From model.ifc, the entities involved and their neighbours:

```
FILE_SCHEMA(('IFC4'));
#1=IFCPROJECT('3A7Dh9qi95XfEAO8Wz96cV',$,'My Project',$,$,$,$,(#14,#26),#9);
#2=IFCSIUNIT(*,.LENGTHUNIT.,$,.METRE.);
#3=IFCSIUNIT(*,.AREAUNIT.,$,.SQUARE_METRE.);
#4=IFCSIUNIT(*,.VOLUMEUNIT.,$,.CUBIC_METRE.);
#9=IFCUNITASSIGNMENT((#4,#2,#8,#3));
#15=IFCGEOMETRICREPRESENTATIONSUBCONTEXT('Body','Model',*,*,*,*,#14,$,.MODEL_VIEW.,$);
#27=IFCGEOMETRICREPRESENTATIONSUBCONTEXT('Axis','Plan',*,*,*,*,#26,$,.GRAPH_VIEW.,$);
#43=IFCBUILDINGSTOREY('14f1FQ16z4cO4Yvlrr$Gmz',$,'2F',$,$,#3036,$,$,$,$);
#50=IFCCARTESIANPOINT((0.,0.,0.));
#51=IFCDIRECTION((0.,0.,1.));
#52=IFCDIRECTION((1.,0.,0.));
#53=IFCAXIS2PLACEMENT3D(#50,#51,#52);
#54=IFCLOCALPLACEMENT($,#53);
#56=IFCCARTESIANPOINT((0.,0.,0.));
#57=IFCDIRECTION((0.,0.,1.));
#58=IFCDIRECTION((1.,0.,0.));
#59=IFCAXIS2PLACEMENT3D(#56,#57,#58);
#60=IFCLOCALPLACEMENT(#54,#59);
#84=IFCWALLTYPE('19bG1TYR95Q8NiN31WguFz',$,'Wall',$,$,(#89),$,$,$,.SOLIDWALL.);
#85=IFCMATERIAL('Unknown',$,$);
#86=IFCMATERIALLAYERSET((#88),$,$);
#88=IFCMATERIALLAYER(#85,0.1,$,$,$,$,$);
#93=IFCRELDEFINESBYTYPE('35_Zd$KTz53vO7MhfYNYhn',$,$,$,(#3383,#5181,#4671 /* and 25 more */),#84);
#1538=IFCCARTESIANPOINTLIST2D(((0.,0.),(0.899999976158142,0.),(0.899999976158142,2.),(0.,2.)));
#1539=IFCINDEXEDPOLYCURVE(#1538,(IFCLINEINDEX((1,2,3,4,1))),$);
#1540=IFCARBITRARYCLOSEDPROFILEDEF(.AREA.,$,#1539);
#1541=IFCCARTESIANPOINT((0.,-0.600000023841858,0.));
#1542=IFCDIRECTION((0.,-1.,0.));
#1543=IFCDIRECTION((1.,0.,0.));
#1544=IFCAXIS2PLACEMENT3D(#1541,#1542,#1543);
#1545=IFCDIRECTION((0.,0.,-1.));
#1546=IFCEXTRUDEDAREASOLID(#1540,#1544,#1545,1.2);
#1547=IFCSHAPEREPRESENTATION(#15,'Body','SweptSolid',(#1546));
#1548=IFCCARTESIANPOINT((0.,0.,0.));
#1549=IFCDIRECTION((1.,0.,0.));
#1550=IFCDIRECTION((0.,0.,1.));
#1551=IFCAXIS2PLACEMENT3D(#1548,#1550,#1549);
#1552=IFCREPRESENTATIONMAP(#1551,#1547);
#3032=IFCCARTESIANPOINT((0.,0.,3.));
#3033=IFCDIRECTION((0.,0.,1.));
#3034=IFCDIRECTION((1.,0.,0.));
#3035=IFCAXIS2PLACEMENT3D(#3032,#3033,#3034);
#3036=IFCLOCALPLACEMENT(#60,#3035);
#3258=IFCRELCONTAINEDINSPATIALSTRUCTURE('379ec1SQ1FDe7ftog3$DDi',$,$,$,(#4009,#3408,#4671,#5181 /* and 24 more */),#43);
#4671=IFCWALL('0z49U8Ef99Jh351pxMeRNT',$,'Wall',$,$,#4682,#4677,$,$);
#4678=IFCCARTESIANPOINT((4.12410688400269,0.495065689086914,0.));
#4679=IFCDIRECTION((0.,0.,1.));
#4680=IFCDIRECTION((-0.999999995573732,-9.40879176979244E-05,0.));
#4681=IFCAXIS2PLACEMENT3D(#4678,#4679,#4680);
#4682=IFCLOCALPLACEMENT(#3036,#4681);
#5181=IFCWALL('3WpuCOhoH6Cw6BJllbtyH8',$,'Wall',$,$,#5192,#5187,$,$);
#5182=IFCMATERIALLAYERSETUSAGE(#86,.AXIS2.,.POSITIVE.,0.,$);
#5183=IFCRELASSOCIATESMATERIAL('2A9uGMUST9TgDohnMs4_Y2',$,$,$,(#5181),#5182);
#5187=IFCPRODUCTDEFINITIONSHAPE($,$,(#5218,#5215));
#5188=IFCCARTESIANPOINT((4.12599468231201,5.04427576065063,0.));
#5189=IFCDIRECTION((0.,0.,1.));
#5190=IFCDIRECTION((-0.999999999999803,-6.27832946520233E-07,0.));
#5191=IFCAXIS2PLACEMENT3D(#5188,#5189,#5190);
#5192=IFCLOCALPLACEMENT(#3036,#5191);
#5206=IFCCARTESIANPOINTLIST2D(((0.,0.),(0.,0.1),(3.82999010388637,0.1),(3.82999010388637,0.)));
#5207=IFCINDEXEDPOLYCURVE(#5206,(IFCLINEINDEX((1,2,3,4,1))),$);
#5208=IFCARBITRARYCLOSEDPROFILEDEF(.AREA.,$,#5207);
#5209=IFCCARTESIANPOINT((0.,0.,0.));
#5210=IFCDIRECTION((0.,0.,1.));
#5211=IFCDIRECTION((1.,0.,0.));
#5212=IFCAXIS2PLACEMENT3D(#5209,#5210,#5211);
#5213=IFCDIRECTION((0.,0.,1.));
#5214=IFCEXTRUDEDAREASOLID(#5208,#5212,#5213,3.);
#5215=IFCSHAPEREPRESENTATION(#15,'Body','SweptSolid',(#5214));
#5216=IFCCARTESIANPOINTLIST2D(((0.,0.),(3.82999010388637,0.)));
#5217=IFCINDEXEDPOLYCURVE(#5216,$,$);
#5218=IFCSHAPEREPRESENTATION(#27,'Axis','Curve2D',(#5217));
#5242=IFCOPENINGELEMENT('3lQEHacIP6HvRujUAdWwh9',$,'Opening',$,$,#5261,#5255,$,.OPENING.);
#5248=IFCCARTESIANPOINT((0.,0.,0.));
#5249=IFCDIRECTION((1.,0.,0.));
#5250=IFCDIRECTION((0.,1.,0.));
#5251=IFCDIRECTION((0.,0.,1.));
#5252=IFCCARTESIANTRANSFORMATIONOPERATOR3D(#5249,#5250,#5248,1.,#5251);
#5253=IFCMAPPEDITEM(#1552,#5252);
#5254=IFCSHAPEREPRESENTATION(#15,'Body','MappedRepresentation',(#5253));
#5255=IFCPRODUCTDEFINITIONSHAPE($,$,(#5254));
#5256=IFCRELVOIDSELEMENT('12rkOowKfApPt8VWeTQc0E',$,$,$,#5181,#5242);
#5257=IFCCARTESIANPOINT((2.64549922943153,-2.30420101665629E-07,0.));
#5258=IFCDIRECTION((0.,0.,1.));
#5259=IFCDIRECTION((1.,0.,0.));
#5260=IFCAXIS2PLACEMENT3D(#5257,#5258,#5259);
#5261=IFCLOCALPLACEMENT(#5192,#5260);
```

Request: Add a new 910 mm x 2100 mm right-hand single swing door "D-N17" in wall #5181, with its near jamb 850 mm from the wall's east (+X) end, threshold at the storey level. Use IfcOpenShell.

```python
import numpy as np
import ifcopenshell
import ifcopenshell.api.feature
import ifcopenshell.api.geometry
import ifcopenshell.api.root
import ifcopenshell.api.spatial
import ifcopenshell.geom
import ifcopenshell.util.element
import ifcopenshell.util.placement
import ifcopenshell.util.representation
import ifcopenshell.util.shape
import ifcopenshell.util.unit

model = ifcopenshell.open("model.ifc")
unit_scale = ifcopenshell.util.unit.calculate_unit_scale(model)
settings = ifcopenshell.geom.settings()


def volume(element):
    """Net volume in cubic metres, openings subtracted."""
    shape = ifcopenshell.geom.create_shape(settings, element)
    return ifcopenshell.util.shape.get_volume(shape.geometry)


wall = model.by_guid("3WpuCOhoH6Cw6BJllbtyH8")
storey = ifcopenshell.util.element.get_container(wall, ifc_class="IfcBuildingStorey")
context = ifcopenshell.util.representation.get_context(model, "Model", "Body", "MODEL_VIEW")
before = volume(wall)

width, height, from_end, sill = 0.91, 2.1, 0.85, 0.0  # metres

# The wall runs along its own X axis, and the end named is its -X end.
wall_shape = ifcopenshell.geom.create_shape(settings, wall)
x, y, z = ifcopenshell.util.shape.get_vertices(wall_shape.geometry).T
start = x.min() + from_end
face, thickness = float(y.min()), float(y.max() - y.min())
wall_matrix = ifcopenshell.util.placement.get_local_placement(wall.ObjectPlacement)
level = ifcopenshell.util.placement.get_local_placement(storey.ObjectPlacement)[2, 3]


def in_wall(x, y):
    """Placement at x, y metres in the wall's axes, at sill height."""
    matrix = wall_matrix.copy()
    matrix[:, 3] = wall_matrix @ np.array([x / unit_scale, y / unit_scale, 0.0, 1.0])
    matrix[2, 3] = level + sill / unit_scale
    return matrix


# Opening: a box that overshoots both wall faces by 50 mm.
opening = ifcopenshell.api.root.create_entity(model, ifc_class="IfcOpeningElement", predefined_type="OPENING")
box = ifcopenshell.api.geometry.add_wall_representation(
    model, context=context, length=width, height=height, thickness=thickness + 0.1
)
ifcopenshell.api.geometry.assign_representation(model, product=opening, representation=box)
ifcopenshell.api.geometry.edit_object_placement(model, product=opening, matrix=in_wall(start, face - 0.05), is_si=False)
ifcopenshell.api.feature.add_feature(model, feature=opening, element=wall)

door = ifcopenshell.api.root.create_entity(model, ifc_class="IfcDoor", name="D-N17", predefined_type="DOOR")
door.OverallWidth, door.OverallHeight = width / unit_scale, height / unit_scale
door.OperationType = "SINGLE_SWING_RIGHT"
body = ifcopenshell.api.geometry.add_door_representation(
    model,
    context=context,
    overall_width=door.OverallWidth,
    overall_height=door.OverallHeight,
    operation_type="SINGLE_SWING_RIGHT",
    lining_properties={"LiningDepth": thickness / unit_scale, "ThresholdDepth": thickness / unit_scale},
)
ifcopenshell.api.geometry.assign_representation(model, product=door, representation=body)
ifcopenshell.api.spatial.assign_container(model, products=[door], relating_structure=storey)
ifcopenshell.api.feature.add_filling(model, opening=opening, element=door)

# The lining spans the wall, so the door starts at the wall face.
ifcopenshell.api.geometry.edit_object_placement(model, product=door, matrix=in_wall(start, face), is_si=False)

after = volume(wall)

print(f"wall volume {before:.3f} -> {after:.3f} m3")

model.write("model_v2.ifc")
```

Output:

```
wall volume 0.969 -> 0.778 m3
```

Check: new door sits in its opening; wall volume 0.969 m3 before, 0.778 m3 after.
